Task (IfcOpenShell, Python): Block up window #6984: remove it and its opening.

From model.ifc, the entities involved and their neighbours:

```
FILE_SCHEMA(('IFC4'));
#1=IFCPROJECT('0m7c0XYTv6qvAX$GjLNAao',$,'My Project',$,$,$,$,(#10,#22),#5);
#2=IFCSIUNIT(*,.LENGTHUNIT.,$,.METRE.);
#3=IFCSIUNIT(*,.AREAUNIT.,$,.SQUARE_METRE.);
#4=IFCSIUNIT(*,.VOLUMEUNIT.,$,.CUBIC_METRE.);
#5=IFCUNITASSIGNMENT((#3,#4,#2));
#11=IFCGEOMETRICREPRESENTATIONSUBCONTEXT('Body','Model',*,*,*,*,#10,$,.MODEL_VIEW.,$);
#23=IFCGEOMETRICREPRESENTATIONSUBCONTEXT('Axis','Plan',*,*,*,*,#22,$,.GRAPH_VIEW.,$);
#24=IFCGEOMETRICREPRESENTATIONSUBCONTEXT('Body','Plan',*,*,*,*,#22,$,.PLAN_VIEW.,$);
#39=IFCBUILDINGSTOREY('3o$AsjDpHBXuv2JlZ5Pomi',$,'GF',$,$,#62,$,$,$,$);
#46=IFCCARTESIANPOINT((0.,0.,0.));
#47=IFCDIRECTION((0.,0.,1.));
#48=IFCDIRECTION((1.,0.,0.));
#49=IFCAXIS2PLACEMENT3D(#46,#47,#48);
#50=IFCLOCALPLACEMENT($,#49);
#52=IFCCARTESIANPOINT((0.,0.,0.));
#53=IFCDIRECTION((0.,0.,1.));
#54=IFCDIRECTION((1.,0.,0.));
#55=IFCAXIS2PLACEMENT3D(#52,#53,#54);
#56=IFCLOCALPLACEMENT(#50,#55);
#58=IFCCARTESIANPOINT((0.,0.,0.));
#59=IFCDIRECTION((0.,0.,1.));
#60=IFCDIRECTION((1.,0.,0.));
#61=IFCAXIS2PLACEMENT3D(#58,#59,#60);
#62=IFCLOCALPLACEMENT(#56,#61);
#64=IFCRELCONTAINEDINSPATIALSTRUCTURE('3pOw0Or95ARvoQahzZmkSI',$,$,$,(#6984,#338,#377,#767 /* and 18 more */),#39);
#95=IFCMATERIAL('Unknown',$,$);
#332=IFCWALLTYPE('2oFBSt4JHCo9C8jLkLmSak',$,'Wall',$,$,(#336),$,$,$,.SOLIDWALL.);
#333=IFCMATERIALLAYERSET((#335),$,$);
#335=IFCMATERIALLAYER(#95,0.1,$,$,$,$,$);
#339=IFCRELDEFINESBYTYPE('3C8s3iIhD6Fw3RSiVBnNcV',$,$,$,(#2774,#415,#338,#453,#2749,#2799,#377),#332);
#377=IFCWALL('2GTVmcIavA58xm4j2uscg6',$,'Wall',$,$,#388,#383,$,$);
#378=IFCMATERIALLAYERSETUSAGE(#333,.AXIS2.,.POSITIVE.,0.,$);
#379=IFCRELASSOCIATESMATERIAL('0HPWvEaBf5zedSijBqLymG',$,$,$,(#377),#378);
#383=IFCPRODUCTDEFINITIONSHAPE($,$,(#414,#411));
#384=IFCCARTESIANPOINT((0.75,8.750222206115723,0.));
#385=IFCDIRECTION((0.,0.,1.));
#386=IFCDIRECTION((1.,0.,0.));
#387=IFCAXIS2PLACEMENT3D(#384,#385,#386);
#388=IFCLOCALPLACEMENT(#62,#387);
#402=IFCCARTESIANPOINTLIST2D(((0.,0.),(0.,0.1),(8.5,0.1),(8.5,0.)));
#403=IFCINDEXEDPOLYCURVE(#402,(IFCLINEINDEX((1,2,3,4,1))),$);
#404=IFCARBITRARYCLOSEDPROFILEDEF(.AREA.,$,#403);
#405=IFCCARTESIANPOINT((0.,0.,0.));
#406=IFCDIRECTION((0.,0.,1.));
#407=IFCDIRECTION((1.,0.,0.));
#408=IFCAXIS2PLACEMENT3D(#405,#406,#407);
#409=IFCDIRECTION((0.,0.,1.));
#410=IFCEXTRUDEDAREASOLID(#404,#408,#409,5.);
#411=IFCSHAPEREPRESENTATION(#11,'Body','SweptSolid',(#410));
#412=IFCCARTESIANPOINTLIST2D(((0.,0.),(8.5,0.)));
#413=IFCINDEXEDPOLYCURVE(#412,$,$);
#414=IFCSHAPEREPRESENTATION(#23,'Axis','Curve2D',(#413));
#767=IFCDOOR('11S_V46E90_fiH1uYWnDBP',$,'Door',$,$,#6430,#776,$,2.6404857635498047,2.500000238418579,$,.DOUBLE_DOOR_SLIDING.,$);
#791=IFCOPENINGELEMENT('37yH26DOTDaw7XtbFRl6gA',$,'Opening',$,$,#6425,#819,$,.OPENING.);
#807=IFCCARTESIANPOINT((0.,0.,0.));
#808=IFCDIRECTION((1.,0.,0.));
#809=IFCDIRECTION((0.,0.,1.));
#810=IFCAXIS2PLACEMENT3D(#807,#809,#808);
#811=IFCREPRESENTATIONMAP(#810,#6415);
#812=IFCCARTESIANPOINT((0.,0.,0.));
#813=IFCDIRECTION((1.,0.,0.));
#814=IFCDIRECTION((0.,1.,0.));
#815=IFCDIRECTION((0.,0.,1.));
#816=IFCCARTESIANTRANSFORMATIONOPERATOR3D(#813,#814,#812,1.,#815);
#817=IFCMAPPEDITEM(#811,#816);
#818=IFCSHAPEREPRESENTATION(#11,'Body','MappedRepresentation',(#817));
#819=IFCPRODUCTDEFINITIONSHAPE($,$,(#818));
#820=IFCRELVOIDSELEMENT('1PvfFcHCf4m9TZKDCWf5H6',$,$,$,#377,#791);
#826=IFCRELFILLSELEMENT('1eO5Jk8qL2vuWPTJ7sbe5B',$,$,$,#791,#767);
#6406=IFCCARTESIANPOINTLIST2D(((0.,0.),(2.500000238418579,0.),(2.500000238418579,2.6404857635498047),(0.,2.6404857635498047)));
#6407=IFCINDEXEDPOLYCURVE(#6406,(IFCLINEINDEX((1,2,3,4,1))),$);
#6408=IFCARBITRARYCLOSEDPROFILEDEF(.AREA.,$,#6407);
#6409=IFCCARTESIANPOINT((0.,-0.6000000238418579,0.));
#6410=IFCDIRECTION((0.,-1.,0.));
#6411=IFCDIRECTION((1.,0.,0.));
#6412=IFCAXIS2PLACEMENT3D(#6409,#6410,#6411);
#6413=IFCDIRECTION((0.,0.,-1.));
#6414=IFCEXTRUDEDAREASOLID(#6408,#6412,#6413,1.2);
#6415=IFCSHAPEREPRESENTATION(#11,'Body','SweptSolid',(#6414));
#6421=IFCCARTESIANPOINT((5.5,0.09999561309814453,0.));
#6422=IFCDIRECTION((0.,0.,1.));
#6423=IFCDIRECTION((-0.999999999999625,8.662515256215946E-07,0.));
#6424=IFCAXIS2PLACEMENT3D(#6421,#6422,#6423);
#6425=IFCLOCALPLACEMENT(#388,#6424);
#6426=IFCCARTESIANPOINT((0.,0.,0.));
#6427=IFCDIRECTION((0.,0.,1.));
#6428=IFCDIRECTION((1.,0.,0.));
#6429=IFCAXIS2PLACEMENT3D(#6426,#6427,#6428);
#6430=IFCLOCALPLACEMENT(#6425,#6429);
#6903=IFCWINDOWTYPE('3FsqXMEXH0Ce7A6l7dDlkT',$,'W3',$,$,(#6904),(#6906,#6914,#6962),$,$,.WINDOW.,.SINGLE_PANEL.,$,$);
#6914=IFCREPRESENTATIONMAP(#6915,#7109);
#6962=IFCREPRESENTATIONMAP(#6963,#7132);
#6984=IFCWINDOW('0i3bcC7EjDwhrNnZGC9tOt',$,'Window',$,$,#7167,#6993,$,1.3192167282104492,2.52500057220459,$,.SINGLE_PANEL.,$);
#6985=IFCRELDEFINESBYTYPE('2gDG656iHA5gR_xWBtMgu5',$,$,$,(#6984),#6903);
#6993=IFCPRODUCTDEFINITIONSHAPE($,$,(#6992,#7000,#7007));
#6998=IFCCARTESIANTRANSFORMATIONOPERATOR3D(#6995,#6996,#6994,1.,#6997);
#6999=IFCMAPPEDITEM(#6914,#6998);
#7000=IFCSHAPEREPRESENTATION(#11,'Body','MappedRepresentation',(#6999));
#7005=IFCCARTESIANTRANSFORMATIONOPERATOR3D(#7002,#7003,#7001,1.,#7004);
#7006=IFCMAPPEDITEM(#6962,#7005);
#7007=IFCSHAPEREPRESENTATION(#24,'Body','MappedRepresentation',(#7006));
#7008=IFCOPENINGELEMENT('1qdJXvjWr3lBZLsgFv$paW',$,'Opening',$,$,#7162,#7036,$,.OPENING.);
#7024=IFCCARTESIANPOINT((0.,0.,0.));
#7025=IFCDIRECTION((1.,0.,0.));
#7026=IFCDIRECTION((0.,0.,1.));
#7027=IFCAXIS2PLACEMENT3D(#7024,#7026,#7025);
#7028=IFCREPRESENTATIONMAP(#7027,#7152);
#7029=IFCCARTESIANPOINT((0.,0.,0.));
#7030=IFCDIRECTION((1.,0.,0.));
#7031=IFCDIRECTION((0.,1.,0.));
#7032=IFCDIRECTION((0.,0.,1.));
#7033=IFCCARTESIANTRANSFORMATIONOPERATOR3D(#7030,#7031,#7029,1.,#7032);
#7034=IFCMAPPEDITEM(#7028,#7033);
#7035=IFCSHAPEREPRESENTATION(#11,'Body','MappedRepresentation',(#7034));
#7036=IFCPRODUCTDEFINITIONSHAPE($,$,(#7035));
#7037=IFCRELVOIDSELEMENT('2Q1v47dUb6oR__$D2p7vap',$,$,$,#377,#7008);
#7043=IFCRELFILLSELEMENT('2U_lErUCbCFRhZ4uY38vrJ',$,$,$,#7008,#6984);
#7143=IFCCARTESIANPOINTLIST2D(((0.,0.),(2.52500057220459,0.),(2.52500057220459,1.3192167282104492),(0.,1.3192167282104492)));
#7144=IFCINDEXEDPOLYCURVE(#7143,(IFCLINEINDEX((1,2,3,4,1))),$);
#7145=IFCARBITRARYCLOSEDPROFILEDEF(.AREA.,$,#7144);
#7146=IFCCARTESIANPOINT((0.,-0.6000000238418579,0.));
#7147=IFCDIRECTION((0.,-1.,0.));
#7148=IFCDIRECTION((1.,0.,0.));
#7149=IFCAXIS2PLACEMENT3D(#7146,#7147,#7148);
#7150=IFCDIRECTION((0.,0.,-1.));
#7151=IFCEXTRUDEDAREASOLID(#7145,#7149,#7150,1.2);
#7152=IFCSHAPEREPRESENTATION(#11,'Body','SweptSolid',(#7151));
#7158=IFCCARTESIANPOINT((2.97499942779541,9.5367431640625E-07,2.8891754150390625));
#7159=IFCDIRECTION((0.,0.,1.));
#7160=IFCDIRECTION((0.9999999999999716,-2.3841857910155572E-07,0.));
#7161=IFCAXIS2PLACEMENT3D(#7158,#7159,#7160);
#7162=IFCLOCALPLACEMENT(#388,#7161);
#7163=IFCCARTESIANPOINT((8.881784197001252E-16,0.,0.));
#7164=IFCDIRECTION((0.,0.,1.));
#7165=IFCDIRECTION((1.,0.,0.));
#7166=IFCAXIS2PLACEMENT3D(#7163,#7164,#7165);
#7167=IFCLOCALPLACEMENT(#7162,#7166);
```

```python
import ifcopenshell
import ifcopenshell.api.feature
import ifcopenshell.api.root
import ifcopenshell.geom
import ifcopenshell.util.shape

model = ifcopenshell.open("model.ifc")
settings = ifcopenshell.geom.settings()


def volume(element):
    """Net volume in cubic metres, openings subtracted."""
    shape = ifcopenshell.geom.create_shape(settings, element)
    return ifcopenshell.util.shape.get_volume(shape.geometry)


window = model.by_guid("0i3bcC7EjDwhrNnZGC9tOt")
opening = window.FillsVoids[0].RelatingOpeningElement
wall = opening.VoidsElements[0].RelatingBuildingElement
before = volume(wall)

ifcopenshell.api.root.remove_product(model, product=window)
ifcopenshell.api.feature.remove_feature(model, feature=opening)

after = volume(wall)

print(f"wall volume {before:.3f} -> {after:.3f} m3")

model.write("model_updated.ifc")
```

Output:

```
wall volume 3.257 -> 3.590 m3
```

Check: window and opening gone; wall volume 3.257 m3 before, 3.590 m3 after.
